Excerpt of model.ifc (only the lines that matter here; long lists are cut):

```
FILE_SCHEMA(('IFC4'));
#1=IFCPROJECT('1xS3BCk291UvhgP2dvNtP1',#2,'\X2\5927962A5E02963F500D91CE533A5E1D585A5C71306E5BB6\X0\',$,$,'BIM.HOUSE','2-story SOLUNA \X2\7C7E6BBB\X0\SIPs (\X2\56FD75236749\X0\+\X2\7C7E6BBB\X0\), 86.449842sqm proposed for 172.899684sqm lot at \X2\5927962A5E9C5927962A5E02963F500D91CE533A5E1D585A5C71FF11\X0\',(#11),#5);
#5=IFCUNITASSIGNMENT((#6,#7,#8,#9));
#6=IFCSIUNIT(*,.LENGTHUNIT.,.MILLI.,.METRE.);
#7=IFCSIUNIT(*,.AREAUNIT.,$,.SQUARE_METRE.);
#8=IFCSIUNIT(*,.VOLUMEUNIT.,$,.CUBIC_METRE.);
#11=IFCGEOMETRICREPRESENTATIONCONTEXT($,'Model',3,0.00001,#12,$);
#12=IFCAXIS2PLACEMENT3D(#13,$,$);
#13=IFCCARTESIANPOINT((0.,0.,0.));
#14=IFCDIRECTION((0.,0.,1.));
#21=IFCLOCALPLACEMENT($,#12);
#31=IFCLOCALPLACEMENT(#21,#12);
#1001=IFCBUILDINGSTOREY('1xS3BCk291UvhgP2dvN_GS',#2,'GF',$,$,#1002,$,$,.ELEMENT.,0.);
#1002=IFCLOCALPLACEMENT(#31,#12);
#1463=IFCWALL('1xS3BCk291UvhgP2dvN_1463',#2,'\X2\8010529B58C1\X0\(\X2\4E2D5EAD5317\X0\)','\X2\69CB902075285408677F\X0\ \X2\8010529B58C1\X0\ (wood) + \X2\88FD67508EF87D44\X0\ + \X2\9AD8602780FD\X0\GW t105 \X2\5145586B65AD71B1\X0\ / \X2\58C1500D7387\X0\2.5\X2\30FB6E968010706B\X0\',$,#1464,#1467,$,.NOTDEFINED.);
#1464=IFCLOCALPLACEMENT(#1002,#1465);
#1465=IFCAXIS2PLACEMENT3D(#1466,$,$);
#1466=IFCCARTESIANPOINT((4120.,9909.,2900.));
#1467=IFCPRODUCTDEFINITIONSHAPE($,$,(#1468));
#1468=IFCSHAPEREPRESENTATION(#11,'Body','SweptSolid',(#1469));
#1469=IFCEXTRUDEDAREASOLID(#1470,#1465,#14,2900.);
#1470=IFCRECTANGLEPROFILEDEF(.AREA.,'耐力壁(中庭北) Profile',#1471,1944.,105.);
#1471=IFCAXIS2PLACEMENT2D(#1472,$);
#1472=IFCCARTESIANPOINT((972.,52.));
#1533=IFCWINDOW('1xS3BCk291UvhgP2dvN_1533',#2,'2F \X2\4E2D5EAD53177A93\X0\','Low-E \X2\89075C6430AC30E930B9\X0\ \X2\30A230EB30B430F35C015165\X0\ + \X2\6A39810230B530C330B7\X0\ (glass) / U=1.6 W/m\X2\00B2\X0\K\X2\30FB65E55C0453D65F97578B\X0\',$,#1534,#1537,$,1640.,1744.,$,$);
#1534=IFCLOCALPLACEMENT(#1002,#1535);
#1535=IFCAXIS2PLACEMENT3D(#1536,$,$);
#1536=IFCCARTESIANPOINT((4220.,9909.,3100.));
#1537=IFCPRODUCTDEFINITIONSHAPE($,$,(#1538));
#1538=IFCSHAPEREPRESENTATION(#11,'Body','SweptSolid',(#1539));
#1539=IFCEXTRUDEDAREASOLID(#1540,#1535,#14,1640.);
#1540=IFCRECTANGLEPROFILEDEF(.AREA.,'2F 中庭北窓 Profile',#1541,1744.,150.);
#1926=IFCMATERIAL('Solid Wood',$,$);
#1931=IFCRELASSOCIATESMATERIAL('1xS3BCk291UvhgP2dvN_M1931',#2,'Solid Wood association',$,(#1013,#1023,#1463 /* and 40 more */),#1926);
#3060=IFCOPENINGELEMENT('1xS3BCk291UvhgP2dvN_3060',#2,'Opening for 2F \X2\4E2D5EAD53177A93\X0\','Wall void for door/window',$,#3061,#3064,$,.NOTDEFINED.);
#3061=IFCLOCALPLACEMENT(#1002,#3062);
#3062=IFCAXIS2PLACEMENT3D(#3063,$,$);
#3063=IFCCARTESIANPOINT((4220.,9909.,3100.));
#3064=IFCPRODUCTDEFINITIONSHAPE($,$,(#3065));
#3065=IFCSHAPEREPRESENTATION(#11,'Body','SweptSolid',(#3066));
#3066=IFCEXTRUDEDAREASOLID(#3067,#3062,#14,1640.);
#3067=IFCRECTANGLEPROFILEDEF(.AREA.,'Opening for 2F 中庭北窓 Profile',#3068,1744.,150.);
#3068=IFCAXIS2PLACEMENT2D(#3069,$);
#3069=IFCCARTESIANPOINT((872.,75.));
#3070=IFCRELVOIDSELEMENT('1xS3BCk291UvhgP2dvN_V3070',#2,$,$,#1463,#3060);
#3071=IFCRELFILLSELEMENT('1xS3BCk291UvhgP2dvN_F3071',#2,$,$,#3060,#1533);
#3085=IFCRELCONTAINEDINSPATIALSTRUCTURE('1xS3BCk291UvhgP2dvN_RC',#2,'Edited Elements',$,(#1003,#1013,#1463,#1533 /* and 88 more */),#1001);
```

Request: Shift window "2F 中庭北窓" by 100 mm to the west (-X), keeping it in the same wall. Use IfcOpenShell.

```python
import ifcopenshell
import ifcopenshell.api.geometry
import ifcopenshell.util.placement
import ifcopenshell.util.unit

model = ifcopenshell.open("model.ifc")
unit_scale = ifcopenshell.util.unit.calculate_unit_scale(model)

window = model.by_id(1533)
opening = window.FillsVoids[0].RelatingOpeningElement
wall = opening.VoidsElements[0].RelatingBuildingElement

wall_matrix = ifcopenshell.util.placement.get_local_placement(wall.ObjectPlacement)
shift = wall_matrix[:3, 0] * -0.1 / unit_scale
before = ifcopenshell.util.placement.get_local_placement(window.ObjectPlacement)[:3, 3].copy()

# The window is not placed relative to its opening, so move both.
for product in (opening, window):
    matrix = ifcopenshell.util.placement.get_local_placement(product.ObjectPlacement)
    matrix[:3, 3] += shift
    ifcopenshell.api.geometry.edit_object_placement(model, product=product, matrix=matrix, is_si=False)

after = ifcopenshell.util.placement.get_local_placement(window.ObjectPlacement)[:3, 3]
print("window moved by", (after - before).round(3) + 0.0)

model.write("model_rev.ifc")
```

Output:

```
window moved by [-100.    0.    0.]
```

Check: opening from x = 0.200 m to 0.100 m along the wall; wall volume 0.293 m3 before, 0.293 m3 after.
